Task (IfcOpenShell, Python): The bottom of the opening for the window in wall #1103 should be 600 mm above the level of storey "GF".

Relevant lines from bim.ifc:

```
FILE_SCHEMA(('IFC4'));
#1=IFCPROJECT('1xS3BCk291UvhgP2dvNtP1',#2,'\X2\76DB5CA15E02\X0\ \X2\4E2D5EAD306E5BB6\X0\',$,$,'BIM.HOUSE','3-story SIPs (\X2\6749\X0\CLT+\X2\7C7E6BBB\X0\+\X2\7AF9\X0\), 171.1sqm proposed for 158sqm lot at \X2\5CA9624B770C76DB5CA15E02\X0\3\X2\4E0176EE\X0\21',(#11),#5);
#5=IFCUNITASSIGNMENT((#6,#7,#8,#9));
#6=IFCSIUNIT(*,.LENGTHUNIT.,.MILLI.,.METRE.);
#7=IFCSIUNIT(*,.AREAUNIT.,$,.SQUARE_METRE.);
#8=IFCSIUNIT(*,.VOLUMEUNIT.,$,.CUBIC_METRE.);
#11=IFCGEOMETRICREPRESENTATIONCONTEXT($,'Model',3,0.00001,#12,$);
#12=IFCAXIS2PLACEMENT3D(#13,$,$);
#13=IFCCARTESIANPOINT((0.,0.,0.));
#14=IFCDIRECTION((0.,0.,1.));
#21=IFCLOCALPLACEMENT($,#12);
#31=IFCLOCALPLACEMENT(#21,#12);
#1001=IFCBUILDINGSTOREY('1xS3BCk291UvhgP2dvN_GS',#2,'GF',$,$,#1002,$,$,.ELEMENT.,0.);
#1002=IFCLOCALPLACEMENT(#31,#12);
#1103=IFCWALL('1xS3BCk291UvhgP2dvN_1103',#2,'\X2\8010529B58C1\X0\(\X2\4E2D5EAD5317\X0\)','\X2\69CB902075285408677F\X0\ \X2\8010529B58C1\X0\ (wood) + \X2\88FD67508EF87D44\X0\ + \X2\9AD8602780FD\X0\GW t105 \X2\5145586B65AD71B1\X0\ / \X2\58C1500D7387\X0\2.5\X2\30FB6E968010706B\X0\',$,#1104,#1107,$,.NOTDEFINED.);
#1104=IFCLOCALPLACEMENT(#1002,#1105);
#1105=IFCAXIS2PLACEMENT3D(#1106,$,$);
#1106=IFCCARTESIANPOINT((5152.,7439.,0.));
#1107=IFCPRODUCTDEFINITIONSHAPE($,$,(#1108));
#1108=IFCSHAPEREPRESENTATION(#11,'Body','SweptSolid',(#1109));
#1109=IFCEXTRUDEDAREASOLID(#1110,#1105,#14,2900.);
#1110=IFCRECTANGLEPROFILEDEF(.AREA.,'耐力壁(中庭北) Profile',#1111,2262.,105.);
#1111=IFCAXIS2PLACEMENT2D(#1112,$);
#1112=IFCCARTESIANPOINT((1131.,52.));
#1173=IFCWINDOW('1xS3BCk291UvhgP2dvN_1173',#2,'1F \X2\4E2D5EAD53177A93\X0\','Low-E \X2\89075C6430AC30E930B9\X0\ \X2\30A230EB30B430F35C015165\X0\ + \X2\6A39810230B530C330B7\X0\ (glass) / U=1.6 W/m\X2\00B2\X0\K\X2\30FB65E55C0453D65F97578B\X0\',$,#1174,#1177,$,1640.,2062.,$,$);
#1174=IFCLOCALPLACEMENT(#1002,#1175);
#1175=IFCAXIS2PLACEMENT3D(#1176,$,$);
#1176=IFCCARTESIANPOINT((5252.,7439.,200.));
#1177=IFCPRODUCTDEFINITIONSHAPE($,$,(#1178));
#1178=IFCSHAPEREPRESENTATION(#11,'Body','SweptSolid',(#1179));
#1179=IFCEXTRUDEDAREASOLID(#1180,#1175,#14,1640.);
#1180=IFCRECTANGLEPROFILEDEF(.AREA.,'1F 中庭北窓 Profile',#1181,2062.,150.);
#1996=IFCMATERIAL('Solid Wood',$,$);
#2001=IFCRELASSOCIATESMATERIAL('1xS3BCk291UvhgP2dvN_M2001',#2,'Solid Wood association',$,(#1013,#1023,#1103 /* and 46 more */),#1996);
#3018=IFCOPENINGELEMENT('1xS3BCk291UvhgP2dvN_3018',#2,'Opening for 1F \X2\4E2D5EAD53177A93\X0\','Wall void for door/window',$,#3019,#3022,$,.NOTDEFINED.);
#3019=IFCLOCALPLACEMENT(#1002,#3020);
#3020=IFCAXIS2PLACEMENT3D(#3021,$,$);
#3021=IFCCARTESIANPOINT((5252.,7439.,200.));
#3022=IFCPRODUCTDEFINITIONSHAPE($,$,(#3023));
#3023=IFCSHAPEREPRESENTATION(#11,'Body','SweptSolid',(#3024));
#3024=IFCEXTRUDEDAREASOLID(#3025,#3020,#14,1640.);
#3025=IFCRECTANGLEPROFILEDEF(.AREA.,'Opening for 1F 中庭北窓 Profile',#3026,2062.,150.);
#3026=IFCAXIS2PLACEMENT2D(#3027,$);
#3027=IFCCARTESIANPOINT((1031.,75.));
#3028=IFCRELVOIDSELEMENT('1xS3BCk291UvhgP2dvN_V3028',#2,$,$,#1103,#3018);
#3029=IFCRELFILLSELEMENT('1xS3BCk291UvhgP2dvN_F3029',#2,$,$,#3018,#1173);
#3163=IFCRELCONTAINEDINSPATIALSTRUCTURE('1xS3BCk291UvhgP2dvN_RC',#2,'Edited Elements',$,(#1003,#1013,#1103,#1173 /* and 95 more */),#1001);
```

```python
import numpy as np
import ifcopenshell
import ifcopenshell.api.geometry
import ifcopenshell.geom
import ifcopenshell.util.element
import ifcopenshell.util.placement
import ifcopenshell.util.shape
import ifcopenshell.util.unit

model = ifcopenshell.open("bim.ifc")
unit_scale = ifcopenshell.util.unit.calculate_unit_scale(model)

window = model.by_guid("1xS3BCk291UvhgP2dvN_1173")
opening = window.FillsVoids[0].RelatingOpeningElement
storey = ifcopenshell.util.element.get_container(window, ifc_class="IfcBuildingStorey")
level = ifcopenshell.util.placement.get_local_placement(storey.ObjectPlacement)[2, 3]

# The opening's origin need not be at the sill, so measure its lowest point.
shape = ifcopenshell.geom.create_shape(ifcopenshell.geom.settings(), opening)
bottom = ifcopenshell.util.shape.get_shape_bottom_elevation(shape, shape.geometry) / unit_scale
dz = level + 600.0 - bottom

shift = np.array([0.0, 0.0, dz])
# The window is not placed relative to its opening, so move both.
for product in (opening, window):
    matrix = ifcopenshell.util.placement.get_local_placement(product.ObjectPlacement)
    matrix[:3, 3] += shift
    ifcopenshell.api.geometry.edit_object_placement(model, product=product, matrix=matrix, is_si=False)

print(f"moved by {dz * unit_scale:+.3f} m")

model.write("bim_v2.ifc")
```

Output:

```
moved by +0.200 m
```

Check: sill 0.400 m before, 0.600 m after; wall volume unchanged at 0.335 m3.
